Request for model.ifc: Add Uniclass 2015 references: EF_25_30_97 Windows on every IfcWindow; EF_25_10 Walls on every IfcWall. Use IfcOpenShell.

First a look at what the model holds.

```python
import ifcopenshell

model = ifcopenshell.open("model.ifc")
print(model.schema)
print("classifications:", [c.Name for c in model.by_type("IfcClassification")])
for ifc_class in ("IfcDoor", "IfcRoof", "IfcStair", "IfcWall", "IfcWindow"):
    print(ifc_class, len(model.by_type(ifc_class)))
```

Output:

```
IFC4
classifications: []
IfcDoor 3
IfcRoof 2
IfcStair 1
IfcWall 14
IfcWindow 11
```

```python
import ifcopenshell
import ifcopenshell.api.classification

model = ifcopenshell.open("model.ifc")

system = ifcopenshell.api.classification.add_classification(model, classification="Uniclass 2015")

codes = {
    "IfcWindow": ("EF_25_30_97", "Windows"),
    "IfcWall": ("EF_25_10", "Walls"),
}
for ifc_class, (code, name) in codes.items():
    products = model.by_type(ifc_class)
    ifcopenshell.api.classification.add_reference(
        model, products=products, classification=system, identification=code, name=name
    )
    print(code, len(products))

model.write("model_rev.ifc")
```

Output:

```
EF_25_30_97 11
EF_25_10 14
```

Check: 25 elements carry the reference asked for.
